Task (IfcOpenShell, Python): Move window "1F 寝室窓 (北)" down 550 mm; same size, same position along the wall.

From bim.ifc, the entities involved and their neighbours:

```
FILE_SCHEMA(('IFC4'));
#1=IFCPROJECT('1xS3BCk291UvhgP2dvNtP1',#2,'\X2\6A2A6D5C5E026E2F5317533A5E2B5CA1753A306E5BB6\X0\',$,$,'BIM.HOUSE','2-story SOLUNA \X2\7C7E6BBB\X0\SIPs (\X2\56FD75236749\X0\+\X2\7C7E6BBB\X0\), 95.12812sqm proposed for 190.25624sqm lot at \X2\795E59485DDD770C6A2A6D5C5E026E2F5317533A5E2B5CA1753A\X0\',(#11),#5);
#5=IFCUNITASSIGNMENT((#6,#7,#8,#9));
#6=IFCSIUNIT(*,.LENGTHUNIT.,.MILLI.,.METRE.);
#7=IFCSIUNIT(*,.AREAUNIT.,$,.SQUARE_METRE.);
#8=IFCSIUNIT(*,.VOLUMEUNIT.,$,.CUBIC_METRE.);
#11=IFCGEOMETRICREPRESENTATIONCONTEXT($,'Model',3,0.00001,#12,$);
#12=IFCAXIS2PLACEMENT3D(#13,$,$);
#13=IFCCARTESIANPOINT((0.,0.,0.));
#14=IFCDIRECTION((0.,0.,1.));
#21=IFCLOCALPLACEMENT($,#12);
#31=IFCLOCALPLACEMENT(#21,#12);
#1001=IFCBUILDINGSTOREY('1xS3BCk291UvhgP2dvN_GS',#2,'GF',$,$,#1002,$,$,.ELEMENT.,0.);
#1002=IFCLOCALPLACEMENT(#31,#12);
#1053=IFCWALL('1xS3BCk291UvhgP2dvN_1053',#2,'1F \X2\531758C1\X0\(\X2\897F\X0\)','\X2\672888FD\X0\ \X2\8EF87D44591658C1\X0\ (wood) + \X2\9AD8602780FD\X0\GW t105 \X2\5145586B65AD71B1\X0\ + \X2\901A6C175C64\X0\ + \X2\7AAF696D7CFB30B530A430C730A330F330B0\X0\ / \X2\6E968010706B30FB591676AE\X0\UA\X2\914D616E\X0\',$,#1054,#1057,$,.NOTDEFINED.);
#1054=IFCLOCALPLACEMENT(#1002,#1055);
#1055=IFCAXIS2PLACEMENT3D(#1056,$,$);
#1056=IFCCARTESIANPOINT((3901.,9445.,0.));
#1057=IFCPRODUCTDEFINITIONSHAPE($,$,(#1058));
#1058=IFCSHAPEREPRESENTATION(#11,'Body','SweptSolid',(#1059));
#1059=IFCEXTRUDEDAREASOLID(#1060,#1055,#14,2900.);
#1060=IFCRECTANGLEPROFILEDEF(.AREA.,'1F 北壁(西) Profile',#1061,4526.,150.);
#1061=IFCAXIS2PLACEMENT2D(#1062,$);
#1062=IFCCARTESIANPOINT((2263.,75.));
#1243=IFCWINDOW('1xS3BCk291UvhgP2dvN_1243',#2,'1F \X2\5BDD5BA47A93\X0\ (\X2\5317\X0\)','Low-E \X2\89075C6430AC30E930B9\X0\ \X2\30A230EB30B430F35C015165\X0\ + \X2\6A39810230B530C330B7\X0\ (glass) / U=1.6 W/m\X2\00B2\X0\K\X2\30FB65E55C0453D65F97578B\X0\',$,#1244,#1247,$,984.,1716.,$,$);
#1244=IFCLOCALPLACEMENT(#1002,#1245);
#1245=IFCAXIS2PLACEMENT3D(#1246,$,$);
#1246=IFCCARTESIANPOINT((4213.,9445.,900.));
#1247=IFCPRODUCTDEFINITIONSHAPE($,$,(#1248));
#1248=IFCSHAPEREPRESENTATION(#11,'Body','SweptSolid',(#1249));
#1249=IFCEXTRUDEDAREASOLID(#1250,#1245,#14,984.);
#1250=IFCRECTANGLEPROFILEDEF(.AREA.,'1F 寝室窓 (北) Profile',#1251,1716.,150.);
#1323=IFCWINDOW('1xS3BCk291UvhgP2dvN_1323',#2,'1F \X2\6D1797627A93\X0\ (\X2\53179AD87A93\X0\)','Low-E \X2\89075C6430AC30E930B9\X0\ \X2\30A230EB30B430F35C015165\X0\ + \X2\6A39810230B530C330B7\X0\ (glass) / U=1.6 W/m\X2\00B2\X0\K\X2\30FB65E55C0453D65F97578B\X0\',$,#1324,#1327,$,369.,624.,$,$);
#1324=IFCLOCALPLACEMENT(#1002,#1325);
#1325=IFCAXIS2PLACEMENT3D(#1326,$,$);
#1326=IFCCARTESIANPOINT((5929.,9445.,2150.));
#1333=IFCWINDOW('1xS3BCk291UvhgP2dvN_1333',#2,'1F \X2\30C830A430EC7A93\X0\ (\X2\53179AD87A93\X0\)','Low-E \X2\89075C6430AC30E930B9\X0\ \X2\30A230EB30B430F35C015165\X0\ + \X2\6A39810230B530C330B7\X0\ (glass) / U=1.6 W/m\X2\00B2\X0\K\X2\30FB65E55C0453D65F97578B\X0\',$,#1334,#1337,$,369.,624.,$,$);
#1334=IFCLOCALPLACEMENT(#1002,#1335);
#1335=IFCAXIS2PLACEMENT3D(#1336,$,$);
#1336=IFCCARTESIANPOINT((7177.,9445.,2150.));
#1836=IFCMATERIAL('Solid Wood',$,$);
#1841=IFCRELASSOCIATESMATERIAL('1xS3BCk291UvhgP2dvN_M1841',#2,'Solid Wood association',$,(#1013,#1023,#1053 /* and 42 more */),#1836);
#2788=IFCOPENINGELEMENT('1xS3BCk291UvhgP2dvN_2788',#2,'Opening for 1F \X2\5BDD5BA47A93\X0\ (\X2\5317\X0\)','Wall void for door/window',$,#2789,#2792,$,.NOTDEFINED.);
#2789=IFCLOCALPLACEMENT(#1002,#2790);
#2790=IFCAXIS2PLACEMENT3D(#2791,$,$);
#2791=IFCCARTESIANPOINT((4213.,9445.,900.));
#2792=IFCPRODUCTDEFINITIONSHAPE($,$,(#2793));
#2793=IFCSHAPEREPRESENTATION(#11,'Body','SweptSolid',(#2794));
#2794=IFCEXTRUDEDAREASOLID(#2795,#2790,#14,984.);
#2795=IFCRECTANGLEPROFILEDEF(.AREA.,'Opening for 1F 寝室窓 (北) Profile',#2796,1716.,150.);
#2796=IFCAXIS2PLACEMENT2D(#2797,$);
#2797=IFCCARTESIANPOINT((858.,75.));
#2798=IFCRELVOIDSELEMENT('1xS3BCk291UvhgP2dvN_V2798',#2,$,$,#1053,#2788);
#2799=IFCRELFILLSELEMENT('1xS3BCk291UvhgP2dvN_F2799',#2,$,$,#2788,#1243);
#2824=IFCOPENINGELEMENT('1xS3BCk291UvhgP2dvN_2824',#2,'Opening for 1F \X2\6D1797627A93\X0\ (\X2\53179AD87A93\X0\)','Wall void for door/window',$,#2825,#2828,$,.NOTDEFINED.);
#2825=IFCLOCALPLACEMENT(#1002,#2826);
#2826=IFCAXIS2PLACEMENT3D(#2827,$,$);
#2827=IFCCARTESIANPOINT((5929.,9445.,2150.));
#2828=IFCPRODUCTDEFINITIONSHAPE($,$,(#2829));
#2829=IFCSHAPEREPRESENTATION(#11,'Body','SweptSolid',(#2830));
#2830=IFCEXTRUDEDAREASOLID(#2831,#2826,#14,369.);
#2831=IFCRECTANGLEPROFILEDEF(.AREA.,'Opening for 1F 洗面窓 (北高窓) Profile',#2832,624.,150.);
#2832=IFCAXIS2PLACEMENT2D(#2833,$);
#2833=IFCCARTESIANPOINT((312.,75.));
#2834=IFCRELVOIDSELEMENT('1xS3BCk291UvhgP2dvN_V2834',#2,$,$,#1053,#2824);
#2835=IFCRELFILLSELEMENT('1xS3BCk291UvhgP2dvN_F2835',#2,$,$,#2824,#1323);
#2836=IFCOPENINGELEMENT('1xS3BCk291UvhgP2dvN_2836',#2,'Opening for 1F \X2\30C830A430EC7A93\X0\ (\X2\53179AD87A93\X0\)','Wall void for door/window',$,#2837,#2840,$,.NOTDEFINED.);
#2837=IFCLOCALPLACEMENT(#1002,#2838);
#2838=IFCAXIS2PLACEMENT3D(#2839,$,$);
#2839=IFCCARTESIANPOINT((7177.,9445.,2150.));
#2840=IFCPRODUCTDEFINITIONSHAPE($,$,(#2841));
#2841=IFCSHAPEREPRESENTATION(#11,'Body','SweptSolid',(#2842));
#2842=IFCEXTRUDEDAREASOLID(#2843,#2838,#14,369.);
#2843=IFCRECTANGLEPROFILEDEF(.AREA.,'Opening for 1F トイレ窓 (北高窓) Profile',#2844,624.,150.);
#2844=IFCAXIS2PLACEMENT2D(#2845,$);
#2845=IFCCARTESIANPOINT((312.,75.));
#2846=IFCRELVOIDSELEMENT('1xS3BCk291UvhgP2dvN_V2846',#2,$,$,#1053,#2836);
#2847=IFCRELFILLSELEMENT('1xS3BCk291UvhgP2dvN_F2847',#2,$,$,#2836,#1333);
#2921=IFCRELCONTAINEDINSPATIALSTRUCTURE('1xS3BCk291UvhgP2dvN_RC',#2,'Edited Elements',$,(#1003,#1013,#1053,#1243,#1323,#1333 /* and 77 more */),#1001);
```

```python
import numpy as np
import ifcopenshell
import ifcopenshell.api.geometry
import ifcopenshell.util.placement
import ifcopenshell.util.unit

model = ifcopenshell.open("bim.ifc")
unit_scale = ifcopenshell.util.unit.calculate_unit_scale(model)

window = model.by_guid("1xS3BCk291UvhgP2dvN_1243")
opening = window.FillsVoids[0].RelatingOpeningElement
dz = -550.0

shift = np.array([0.0, 0.0, dz])
# The window is not placed relative to its opening, so move both.
for product in (opening, window):
    matrix = ifcopenshell.util.placement.get_local_placement(product.ObjectPlacement)
    matrix[:3, 3] += shift
    ifcopenshell.api.geometry.edit_object_placement(model, product=product, matrix=matrix, is_si=False)

print(f"moved by {dz * unit_scale:+.3f} m")

model.write("bim_edited.ifc")
```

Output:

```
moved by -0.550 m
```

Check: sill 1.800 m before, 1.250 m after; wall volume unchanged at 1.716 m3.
